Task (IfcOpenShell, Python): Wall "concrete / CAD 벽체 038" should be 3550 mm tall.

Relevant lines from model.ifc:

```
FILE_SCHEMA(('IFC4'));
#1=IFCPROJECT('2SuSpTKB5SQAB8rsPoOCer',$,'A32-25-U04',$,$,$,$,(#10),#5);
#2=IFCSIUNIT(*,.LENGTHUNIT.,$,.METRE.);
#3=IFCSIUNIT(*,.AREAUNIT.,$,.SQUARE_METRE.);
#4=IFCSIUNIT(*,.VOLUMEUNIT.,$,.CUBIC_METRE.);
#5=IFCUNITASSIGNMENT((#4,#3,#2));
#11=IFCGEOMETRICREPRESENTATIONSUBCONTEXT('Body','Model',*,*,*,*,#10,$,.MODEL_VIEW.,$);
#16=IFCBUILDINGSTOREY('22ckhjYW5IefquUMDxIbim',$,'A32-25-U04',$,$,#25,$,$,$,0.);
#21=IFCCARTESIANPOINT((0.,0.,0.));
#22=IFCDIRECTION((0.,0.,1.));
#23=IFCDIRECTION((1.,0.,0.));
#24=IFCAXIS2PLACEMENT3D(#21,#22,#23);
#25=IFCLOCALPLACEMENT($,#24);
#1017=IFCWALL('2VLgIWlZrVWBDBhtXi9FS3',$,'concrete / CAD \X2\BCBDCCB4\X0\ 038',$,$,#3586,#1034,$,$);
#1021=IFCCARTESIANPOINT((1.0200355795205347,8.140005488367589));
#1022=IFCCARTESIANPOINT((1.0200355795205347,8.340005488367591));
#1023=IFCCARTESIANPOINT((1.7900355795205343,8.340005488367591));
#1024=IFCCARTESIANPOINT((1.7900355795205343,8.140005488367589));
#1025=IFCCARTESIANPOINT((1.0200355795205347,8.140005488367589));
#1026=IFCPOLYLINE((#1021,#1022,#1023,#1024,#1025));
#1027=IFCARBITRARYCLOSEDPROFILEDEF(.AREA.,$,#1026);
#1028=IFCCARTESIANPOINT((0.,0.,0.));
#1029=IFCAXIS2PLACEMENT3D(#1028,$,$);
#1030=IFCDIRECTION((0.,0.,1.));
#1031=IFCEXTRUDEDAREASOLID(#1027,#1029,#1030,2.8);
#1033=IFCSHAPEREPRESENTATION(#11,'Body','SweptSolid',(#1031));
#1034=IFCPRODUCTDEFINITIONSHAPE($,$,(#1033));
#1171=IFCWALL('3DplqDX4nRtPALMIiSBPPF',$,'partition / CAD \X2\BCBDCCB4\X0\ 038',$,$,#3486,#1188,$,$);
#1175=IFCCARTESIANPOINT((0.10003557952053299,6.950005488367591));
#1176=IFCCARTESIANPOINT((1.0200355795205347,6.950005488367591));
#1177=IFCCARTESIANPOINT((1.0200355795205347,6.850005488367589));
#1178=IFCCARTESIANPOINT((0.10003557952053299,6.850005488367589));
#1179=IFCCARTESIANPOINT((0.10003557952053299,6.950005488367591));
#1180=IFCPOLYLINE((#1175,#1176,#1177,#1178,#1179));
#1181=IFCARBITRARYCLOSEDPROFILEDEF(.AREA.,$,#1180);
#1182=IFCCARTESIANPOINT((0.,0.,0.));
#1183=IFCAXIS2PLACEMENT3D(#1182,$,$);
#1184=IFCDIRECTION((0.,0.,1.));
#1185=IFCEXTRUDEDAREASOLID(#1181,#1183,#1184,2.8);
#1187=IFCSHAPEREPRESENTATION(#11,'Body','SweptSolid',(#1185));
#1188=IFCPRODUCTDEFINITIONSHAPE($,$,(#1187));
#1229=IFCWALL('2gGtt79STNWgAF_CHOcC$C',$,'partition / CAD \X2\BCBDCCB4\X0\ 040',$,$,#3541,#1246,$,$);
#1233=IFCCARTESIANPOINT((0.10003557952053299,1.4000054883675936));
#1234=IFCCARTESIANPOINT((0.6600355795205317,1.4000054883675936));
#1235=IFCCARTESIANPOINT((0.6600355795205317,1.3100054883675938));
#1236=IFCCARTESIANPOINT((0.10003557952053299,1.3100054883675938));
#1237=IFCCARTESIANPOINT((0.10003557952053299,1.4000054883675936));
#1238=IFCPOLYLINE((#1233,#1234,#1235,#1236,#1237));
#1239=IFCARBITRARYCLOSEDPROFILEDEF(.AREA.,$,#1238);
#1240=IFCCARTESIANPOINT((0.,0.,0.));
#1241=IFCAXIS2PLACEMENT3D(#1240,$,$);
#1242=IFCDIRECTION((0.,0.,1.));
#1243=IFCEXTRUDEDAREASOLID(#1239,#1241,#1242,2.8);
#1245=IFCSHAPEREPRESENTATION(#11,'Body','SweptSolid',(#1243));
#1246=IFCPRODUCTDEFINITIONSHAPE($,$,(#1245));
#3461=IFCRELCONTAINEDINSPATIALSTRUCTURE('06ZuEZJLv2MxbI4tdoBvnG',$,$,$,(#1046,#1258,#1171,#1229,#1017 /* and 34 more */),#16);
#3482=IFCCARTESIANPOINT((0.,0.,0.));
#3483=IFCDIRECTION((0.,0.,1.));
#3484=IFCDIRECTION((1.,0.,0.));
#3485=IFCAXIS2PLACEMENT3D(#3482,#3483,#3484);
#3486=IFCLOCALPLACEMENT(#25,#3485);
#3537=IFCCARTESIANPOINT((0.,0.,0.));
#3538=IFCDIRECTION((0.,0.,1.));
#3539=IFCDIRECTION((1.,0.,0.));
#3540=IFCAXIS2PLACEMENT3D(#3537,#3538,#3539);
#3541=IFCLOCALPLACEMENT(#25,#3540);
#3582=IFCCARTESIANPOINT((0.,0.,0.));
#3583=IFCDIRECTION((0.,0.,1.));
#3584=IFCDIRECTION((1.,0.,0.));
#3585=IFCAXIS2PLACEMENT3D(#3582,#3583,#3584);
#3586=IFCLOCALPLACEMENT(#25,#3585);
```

```python
import ifcopenshell
import ifcopenshell.geom
import ifcopenshell.util.representation
import ifcopenshell.util.shape

model = ifcopenshell.open("model.ifc")
settings = ifcopenshell.geom.settings()


def volume(element):
    """Net volume in cubic metres, openings subtracted."""
    shape = ifcopenshell.geom.create_shape(settings, element)
    return ifcopenshell.util.shape.get_volume(shape.geometry)


wall = model.by_guid("2VLgIWlZrVWBDBhtXi9FS3")
before = volume(wall)

body = ifcopenshell.util.representation.get_representation(wall, "Model", "Body")
solid = body.Items[0]
old_height = solid.Depth
solid.Depth = 3.55
after = volume(wall)

print(f"height {old_height:g} -> {solid.Depth:g}, volume {before:.3f} -> {after:.3f} m3")

model.write("model-out.ifc")
```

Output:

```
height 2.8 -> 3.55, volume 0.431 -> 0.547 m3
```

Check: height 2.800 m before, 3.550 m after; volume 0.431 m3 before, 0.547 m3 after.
